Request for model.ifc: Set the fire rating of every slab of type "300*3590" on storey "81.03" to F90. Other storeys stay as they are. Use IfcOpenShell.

First a look at what the model holds.

```python
import ifcopenshell
import ifcopenshell.util.element

model = ifcopenshell.open("model.ifc")
print(model.schema)
storey = next(s for s in model.by_type("IfcBuildingStorey") if s.Name == "81.03")
slabs = [e for e in ifcopenshell.util.element.get_decomposition(storey) if e.is_a("IfcSlab")]
seen = {}
for e in slabs:
    element_type = ifcopenshell.util.element.get_type(e)
    key = (element_type.Name if element_type != e and element_type else None, ifcopenshell.util.element.get_pset(e, "Pset_SlabCommon", "FireRating"))
    seen[key] = seen.get(key, 0) + 1
for (name, value), count in sorted(seen.items(), key=str):
    print(count, "x", name, "|", value)
```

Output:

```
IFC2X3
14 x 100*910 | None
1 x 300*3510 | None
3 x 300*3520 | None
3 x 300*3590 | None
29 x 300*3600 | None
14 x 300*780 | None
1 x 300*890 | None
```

```python
import ifcopenshell
import ifcopenshell.api.pset
import ifcopenshell.util.element

model = ifcopenshell.open("model.ifc")

storey = next(s for s in model.by_type("IfcBuildingStorey") if s.Name == "81.03")
slabs = [e for e in ifcopenshell.util.element.get_decomposition(storey) if e.is_a("IfcSlab")]

count = 0
for e in slabs:
    element_type = ifcopenshell.util.element.get_type(e)
    if element_type in (None, e) or element_type.Name != "300*3590":
        continue
    found = ifcopenshell.util.element.get_pset(e, "Pset_SlabCommon", should_inherit=False)
    if found:
        pset = model.by_id(found["id"])
        if len(ifcopenshell.util.element.get_elements_by_pset(pset)) > 1:
            pset = ifcopenshell.api.pset.unshare_pset(model, products=[e], pset=pset)[0]
    else:
        pset = ifcopenshell.api.pset.add_pset(model, product=e, name="Pset_SlabCommon")
    ifcopenshell.api.pset.edit_pset(model, pset=pset, properties={"FireRating": "F90"})
    count += 1

print(count, "slabs updated")

model.write("model-out.ifc")
```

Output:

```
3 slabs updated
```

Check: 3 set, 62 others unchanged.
